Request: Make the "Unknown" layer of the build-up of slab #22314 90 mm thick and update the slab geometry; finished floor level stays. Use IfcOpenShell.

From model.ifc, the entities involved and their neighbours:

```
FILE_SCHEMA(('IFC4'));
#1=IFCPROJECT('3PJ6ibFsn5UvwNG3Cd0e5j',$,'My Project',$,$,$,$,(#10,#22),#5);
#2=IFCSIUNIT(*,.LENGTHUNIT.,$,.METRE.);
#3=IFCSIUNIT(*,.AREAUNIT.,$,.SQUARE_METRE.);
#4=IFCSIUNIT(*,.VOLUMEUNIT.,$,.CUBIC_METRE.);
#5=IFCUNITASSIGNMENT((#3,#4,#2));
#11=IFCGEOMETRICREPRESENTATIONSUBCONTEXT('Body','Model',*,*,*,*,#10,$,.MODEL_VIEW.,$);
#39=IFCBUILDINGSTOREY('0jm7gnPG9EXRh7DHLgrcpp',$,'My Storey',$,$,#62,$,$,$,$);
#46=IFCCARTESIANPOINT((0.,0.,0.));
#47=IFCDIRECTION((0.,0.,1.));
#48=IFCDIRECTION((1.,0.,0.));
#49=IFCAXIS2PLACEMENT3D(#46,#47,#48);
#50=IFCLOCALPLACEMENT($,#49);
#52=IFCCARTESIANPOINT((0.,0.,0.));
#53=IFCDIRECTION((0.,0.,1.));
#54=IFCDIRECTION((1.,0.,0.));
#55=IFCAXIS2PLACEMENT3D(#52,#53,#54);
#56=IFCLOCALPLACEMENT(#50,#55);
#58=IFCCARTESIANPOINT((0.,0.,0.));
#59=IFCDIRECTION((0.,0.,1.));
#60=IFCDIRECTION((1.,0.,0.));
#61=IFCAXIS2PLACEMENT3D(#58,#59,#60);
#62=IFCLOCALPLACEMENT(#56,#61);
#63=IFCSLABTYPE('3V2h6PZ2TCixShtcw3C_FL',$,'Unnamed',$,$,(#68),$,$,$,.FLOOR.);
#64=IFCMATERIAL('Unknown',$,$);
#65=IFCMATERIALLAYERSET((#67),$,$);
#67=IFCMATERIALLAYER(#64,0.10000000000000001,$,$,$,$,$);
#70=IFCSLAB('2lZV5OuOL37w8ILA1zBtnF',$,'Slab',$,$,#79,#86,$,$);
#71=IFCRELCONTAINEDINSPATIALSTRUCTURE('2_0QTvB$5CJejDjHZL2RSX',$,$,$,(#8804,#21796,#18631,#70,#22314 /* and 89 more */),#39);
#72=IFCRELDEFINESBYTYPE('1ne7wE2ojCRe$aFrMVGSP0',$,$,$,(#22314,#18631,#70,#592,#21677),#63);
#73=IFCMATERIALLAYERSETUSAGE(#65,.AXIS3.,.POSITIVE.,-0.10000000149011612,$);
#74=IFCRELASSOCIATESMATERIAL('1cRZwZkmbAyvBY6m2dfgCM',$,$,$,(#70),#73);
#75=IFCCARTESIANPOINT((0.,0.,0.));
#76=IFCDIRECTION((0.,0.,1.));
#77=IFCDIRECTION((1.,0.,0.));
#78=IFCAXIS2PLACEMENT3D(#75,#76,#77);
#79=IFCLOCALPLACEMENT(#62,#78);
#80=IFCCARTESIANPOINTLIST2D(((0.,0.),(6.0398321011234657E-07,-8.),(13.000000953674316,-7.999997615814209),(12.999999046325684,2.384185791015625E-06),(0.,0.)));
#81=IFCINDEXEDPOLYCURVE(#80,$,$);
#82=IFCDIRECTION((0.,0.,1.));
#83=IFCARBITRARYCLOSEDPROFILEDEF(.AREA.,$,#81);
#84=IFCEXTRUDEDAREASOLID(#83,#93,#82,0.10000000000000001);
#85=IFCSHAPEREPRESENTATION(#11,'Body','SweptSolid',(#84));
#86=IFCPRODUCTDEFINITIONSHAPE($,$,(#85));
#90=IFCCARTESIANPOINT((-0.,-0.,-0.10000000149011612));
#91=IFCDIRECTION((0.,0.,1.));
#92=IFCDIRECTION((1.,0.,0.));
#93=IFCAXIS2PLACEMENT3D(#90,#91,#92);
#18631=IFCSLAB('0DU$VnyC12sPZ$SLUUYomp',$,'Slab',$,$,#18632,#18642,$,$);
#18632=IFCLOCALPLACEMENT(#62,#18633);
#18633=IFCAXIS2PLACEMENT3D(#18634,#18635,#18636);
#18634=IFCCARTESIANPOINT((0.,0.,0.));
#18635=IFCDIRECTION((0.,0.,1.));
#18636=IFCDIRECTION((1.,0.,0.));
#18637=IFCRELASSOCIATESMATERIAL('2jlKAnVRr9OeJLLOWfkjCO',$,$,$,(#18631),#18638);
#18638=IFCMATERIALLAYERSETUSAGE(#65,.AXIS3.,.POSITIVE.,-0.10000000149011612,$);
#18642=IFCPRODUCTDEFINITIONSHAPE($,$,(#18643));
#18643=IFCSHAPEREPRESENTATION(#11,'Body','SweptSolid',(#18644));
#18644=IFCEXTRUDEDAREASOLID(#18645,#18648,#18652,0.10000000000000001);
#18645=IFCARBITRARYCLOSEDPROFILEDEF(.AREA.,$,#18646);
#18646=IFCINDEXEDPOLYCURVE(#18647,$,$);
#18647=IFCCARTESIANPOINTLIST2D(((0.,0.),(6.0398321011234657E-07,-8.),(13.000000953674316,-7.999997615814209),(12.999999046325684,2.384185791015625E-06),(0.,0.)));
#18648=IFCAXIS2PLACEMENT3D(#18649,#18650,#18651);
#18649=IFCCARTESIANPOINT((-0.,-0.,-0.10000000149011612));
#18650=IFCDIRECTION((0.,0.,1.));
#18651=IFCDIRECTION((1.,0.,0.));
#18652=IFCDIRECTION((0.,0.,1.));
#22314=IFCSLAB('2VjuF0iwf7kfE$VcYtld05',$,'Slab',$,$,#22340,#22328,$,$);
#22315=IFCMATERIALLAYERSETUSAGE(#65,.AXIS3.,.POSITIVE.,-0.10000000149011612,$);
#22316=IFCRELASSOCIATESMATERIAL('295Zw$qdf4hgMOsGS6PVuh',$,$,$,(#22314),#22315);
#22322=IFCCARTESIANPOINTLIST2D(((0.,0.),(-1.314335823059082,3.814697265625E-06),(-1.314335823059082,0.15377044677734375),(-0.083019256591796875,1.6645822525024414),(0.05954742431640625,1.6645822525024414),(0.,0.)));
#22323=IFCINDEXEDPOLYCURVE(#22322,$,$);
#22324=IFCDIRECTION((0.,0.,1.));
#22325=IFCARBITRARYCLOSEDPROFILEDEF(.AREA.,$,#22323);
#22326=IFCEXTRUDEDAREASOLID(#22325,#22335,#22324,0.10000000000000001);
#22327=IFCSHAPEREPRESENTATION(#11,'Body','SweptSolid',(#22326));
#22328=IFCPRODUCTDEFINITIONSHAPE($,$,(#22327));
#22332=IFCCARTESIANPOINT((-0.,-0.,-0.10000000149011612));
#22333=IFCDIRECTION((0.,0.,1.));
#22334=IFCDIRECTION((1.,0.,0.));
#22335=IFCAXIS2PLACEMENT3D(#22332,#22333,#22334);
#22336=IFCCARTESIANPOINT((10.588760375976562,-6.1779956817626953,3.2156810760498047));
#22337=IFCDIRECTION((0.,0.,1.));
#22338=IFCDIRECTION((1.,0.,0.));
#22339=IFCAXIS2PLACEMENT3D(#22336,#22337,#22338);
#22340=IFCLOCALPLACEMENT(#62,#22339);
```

```python
import ifcopenshell
import ifcopenshell.util.element
import ifcopenshell.util.representation
import ifcopenshell.util.unit

model = ifcopenshell.open("model.ifc")
unit_scale = ifcopenshell.util.unit.calculate_unit_scale(model)

layer_set = model.by_id(65)
layer = next(l for l in layer_set.MaterialLayers if l.Material and l.Material.Name == "Unknown")
change = 0.09 / unit_scale - layer.LayerThickness
layer.LayerThickness += change

# The layer set is shared, so every slab that uses it gets the new thickness.
slabs = [e for e in ifcopenshell.util.element.get_elements_by_material(model, layer_set) if e.is_a("IfcSlab")]
for slab in sorted(slabs, key=lambda e: e.id()):
    body = ifcopenshell.util.representation.get_representation(slab, "Model", "Body")
    solid = body.Items[0]
    old_depth = solid.Depth
    solid.Depth += change
    # Extruded upwards: lower the start of the extrusion so the top stays.
    x, y, z = solid.Position.Location.Coordinates
    solid.Position.Location = model.createIfcCartesianPoint((x, y, z - change))
    print(slab.id(), f"{old_depth:g} -> {solid.Depth:g}")

# The layers are counted up from the underside, which has moved.
for usage in {ifcopenshell.util.element.get_material(slab) for slab in slabs}:
    usage.OffsetFromReferenceLine -= change

model.write("model_v2.ifc")
```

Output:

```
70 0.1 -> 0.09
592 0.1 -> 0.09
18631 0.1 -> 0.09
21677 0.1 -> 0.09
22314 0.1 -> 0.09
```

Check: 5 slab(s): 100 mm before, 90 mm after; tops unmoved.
